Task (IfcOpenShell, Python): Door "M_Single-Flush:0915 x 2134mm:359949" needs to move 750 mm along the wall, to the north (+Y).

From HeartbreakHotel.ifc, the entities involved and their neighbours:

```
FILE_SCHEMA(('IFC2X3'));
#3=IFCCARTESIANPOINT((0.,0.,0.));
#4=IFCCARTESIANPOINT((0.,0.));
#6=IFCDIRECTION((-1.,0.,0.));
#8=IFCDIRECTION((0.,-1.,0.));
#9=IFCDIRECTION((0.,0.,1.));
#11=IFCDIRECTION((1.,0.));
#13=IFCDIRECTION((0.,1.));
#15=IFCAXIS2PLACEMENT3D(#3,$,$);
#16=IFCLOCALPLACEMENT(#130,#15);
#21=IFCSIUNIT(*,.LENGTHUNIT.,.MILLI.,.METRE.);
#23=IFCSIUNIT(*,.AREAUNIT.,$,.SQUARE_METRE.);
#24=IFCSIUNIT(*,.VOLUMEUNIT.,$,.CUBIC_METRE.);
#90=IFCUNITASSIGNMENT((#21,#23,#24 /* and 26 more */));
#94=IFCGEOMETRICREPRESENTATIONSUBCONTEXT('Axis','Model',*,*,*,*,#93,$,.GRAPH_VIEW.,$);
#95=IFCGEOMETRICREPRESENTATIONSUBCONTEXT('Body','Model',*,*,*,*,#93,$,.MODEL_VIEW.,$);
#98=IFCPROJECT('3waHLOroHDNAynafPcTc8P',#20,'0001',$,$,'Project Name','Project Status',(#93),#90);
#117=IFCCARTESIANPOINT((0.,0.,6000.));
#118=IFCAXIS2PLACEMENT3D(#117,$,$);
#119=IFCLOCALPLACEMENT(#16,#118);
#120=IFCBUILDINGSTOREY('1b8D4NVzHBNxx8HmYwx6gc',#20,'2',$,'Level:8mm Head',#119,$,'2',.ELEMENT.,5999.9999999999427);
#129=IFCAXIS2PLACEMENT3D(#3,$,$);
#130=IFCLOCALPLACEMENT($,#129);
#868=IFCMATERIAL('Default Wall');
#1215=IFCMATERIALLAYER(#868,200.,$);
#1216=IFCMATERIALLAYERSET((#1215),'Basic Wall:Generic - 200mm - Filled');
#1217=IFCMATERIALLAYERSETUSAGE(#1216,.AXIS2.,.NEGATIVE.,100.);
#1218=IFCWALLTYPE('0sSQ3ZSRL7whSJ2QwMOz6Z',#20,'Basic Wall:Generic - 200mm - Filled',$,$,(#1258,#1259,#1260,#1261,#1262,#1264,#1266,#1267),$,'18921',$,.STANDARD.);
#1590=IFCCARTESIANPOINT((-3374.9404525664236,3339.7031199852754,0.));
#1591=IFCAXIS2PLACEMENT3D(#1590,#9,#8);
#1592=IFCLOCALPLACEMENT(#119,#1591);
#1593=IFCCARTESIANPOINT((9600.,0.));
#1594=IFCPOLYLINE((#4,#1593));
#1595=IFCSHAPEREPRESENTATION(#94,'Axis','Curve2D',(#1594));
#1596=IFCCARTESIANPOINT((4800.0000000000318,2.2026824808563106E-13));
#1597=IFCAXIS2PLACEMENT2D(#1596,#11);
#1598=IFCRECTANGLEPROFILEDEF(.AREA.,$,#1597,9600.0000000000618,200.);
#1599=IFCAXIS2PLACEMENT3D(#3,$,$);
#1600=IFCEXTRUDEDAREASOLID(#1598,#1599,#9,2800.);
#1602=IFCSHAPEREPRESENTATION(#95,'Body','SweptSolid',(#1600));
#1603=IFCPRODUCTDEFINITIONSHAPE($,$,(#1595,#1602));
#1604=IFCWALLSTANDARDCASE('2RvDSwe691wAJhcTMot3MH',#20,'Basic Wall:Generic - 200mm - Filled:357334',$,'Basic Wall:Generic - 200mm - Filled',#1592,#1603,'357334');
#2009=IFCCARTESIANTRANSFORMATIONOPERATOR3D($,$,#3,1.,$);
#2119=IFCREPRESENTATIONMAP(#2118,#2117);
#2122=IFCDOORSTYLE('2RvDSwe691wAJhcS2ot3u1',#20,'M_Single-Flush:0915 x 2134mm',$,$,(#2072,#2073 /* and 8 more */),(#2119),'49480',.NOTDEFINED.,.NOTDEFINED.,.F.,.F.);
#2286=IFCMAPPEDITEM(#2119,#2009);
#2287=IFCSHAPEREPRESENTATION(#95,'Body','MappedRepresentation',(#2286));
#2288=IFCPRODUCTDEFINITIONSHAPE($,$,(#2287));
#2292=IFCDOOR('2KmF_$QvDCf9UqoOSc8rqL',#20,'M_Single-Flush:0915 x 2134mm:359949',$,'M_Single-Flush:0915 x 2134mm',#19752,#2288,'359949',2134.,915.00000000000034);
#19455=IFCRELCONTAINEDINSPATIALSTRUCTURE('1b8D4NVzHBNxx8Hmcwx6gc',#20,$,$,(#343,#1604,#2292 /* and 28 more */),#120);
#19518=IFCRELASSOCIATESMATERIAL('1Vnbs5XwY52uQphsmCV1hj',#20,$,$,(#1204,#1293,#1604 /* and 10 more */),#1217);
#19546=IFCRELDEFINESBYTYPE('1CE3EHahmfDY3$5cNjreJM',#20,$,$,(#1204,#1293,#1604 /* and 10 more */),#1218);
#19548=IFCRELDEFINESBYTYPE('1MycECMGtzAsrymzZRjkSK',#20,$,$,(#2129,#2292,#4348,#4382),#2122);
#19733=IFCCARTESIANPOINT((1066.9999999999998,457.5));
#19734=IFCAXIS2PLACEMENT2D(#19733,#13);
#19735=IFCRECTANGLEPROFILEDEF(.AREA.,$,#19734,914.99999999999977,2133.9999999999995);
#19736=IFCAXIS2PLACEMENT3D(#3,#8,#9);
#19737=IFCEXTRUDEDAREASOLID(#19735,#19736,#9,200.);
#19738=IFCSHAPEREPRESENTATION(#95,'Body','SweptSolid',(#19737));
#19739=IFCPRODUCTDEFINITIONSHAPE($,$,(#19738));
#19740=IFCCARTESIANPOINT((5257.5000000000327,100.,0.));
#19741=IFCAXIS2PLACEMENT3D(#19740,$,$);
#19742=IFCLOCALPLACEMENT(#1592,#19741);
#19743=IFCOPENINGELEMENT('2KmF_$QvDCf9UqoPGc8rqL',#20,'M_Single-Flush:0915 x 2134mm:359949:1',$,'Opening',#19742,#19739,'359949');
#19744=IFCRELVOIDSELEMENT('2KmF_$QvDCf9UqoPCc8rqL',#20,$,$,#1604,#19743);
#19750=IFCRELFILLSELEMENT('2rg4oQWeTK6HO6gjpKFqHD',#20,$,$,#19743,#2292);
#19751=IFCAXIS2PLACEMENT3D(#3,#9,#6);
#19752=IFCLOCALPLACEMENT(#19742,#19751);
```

```python
import ifcopenshell
import ifcopenshell.api.geometry
import ifcopenshell.util.placement

model = ifcopenshell.open("HeartbreakHotel.ifc")

door = model.by_id(2292)
opening = door.FillsVoids[0].RelatingOpeningElement
wall = opening.VoidsElements[0].RelatingBuildingElement

wall_matrix = ifcopenshell.util.placement.get_local_placement(wall.ObjectPlacement)
shift = wall_matrix[:3, 0] * -750.0
before = ifcopenshell.util.placement.get_local_placement(door.ObjectPlacement)[:3, 3].copy()

# The door is placed relative to its opening, so it follows when the opening moves.
matrix = ifcopenshell.util.placement.get_local_placement(opening.ObjectPlacement)
matrix[:3, 3] += shift
ifcopenshell.api.geometry.edit_object_placement(
    model, product=opening, matrix=matrix, is_si=False, should_transform_children=True
)

after = ifcopenshell.util.placement.get_local_placement(door.ObjectPlacement)[:3, 3]
print("door moved by", (after - before).round(3) + 0.0)

model.write("HeartbreakHotel_updated.ifc")
```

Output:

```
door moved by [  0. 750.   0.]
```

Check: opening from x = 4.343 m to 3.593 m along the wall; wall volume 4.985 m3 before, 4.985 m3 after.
